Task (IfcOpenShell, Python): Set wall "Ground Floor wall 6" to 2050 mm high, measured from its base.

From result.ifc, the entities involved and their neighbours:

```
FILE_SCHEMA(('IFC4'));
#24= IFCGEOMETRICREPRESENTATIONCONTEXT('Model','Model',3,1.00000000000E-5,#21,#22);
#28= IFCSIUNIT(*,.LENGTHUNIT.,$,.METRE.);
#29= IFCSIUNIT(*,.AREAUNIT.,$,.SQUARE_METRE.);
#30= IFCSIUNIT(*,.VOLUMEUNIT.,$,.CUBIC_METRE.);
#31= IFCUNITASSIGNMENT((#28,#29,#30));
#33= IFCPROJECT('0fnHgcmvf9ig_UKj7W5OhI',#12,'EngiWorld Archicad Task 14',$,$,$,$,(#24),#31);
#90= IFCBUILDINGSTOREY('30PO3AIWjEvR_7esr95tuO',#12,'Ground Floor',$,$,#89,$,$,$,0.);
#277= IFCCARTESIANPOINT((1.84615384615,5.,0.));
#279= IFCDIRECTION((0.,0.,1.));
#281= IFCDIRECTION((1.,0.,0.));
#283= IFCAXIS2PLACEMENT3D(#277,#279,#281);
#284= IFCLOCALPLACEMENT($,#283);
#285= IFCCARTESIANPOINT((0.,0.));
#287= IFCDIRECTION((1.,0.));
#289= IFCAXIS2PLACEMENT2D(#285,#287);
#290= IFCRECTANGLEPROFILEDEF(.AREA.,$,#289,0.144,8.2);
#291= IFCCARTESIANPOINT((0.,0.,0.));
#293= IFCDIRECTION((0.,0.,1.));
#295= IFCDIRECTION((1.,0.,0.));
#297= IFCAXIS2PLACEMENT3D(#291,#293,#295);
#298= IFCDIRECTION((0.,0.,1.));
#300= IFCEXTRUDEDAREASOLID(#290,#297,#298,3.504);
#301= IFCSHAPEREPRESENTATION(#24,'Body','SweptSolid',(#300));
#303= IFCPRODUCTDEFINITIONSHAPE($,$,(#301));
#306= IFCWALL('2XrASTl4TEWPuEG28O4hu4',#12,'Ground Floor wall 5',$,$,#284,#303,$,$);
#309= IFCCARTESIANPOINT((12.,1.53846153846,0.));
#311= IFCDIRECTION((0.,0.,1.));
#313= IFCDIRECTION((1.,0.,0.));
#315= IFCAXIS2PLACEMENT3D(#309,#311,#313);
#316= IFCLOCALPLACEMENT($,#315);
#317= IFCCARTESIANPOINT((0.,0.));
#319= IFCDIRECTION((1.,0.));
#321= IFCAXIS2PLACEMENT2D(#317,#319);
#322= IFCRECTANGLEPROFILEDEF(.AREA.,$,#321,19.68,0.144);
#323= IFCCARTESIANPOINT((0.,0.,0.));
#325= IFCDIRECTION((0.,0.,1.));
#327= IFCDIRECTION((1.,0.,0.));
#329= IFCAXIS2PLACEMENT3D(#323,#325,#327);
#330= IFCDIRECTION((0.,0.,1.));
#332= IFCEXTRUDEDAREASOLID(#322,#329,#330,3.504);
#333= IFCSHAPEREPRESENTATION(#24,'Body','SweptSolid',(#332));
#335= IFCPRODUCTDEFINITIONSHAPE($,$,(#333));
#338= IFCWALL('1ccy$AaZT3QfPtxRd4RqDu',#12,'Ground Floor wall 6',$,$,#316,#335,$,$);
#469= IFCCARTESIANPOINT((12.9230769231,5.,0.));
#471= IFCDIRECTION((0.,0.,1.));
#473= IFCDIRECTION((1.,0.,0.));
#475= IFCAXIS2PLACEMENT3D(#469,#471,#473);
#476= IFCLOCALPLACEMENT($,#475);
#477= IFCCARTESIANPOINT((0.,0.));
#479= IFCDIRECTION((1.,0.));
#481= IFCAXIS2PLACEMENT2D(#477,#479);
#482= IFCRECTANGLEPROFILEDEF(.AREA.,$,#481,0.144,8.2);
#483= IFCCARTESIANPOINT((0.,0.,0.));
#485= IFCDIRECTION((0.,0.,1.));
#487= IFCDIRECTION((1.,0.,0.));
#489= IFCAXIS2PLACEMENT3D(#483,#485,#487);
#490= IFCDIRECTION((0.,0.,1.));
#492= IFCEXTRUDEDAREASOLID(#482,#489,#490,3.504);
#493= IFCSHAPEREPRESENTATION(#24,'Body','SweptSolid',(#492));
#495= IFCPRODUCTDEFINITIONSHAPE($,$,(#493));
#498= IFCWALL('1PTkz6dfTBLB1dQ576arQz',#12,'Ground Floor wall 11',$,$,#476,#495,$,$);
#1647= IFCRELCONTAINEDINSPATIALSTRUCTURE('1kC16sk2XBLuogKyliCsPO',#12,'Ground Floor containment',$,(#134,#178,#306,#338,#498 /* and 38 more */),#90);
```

```python
import ifcopenshell
import ifcopenshell.geom
import ifcopenshell.util.shape

model = ifcopenshell.open("result.ifc")
settings = ifcopenshell.geom.settings()


def volume(element):
    """Net volume in cubic metres, openings subtracted."""
    shape = ifcopenshell.geom.create_shape(settings, element)
    return ifcopenshell.util.shape.get_volume(shape.geometry)


wall = model.by_guid("1ccy$AaZT3QfPtxRd4RqDu")
before = volume(wall)

body = next(r for r in wall.Representation.Representations if r.RepresentationIdentifier == "Body")
solid = body.Items[0]
old_height = solid.Depth
solid.Depth = 2.05
after = volume(wall)

print(f"height {old_height:g} -> {solid.Depth:g}, volume {before:.3f} -> {after:.3f} m3")

model.write("result_edited.ifc")
```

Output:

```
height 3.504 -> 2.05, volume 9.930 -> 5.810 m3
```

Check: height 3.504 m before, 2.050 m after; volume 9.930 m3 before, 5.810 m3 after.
